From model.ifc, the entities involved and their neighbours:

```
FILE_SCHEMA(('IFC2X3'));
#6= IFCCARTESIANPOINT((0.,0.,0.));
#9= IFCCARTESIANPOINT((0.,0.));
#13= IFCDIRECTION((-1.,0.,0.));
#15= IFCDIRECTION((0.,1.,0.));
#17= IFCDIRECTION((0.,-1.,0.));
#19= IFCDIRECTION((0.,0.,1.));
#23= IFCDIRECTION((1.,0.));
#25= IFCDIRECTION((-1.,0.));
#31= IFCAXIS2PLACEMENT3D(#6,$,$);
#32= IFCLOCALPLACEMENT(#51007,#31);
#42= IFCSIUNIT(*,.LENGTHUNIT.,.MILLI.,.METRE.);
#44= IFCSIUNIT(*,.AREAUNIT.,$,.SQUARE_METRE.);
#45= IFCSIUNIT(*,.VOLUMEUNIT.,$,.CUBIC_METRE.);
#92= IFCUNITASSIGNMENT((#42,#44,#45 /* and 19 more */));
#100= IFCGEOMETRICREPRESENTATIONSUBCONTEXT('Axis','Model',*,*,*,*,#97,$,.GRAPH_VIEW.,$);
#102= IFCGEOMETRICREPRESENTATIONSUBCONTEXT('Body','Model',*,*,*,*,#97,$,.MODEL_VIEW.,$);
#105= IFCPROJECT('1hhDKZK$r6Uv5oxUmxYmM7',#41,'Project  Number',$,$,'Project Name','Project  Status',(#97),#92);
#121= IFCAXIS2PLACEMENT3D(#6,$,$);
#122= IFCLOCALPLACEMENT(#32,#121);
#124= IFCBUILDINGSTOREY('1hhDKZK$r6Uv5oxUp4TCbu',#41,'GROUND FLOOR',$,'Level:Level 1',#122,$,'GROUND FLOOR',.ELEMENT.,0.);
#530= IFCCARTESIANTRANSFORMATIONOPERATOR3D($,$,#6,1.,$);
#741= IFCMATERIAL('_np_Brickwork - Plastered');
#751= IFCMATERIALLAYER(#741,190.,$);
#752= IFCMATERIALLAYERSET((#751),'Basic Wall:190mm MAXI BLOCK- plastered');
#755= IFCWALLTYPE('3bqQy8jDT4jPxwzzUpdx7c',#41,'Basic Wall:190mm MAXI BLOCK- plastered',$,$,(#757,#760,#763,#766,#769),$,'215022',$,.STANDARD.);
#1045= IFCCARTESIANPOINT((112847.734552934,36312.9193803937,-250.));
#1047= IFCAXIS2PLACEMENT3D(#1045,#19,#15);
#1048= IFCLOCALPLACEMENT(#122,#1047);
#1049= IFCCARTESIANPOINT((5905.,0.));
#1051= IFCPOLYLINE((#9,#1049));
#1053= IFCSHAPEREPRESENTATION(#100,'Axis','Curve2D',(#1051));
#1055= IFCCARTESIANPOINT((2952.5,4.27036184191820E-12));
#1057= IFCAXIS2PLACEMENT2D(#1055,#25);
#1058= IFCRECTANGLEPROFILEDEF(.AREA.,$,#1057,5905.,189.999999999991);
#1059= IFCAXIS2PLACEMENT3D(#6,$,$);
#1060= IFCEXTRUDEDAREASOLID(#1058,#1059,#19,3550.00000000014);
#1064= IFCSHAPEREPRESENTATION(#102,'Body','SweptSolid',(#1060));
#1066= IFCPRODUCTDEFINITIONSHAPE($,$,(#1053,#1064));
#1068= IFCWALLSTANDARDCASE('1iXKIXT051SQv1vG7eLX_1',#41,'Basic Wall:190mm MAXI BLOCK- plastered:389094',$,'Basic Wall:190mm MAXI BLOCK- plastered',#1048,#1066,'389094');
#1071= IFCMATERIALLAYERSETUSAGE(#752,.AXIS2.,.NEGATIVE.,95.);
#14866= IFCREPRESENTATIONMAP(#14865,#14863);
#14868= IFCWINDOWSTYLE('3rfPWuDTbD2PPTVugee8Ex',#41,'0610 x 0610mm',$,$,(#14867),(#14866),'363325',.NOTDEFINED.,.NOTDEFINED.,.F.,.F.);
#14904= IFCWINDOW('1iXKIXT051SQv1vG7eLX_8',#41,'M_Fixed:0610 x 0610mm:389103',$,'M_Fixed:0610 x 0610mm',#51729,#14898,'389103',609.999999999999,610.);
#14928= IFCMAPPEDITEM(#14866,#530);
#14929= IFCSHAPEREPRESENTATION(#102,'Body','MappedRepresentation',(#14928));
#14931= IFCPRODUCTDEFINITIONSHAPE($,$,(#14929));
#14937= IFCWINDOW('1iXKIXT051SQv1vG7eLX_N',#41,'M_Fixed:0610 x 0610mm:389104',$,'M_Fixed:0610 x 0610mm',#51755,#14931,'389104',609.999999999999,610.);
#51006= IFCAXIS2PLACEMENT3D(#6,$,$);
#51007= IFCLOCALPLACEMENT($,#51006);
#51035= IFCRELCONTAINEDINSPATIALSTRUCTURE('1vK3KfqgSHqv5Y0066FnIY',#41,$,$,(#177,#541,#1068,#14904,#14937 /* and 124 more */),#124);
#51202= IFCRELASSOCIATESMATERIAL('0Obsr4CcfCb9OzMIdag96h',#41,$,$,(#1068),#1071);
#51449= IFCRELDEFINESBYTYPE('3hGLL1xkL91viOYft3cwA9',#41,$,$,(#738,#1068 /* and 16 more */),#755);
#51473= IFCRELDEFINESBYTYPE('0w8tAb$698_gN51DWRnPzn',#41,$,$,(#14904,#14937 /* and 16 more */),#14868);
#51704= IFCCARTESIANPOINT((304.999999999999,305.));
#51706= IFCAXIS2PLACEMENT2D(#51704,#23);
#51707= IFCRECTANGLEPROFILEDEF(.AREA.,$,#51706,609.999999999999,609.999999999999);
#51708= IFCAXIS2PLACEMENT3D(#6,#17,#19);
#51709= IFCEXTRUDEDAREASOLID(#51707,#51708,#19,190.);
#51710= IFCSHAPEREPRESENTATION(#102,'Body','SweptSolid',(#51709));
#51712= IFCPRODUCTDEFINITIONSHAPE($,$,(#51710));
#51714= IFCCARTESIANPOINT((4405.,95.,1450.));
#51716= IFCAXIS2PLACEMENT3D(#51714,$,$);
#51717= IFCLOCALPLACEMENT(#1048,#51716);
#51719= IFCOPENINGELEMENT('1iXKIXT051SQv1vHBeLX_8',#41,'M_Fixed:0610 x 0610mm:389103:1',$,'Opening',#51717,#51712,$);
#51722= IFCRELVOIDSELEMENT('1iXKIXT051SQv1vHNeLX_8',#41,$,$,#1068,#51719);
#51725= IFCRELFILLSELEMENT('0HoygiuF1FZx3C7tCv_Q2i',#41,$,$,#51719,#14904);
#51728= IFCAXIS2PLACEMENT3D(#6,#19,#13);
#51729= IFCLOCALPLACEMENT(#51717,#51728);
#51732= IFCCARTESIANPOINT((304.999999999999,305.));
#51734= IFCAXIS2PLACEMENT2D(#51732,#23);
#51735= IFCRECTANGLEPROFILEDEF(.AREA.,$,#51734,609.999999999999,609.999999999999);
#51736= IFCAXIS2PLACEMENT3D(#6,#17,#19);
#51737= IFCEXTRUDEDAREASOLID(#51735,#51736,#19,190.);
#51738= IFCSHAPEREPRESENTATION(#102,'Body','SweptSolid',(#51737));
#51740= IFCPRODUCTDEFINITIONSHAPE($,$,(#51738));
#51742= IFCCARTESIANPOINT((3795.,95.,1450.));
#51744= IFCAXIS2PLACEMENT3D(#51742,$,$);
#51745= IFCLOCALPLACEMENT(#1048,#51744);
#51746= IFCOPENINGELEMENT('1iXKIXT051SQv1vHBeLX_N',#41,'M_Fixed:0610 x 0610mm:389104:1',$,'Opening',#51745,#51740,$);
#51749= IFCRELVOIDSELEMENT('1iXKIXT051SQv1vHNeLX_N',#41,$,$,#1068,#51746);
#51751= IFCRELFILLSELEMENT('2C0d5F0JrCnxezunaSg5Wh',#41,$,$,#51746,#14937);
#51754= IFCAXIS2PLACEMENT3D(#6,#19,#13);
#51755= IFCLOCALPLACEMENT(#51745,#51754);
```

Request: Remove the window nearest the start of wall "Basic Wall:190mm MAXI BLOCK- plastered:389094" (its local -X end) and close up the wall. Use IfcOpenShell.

```python
import ifcopenshell
import ifcopenshell.api.feature
import ifcopenshell.api.root
import ifcopenshell.geom
import ifcopenshell.util.shape

model = ifcopenshell.open("model.ifc")
settings = ifcopenshell.geom.settings()


def volume(element):
    """Net volume in cubic metres, openings subtracted."""
    shape = ifcopenshell.geom.create_shape(settings, element)
    return ifcopenshell.util.shape.get_volume(shape.geometry)


window = model.by_guid("1iXKIXT051SQv1vG7eLX_N")
opening = window.FillsVoids[0].RelatingOpeningElement
wall = opening.VoidsElements[0].RelatingBuildingElement
before = volume(wall)

ifcopenshell.api.root.remove_product(model, product=window)
ifcopenshell.api.feature.remove_feature(model, feature=opening)

after = volume(wall)

print(f"wall volume {before:.3f} -> {after:.3f} m3")

model.write("model_rev.ifc")
```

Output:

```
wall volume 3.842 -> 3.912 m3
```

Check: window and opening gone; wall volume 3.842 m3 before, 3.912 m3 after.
